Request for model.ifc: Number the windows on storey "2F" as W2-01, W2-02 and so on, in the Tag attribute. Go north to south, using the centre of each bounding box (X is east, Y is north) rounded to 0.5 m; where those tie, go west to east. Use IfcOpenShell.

First a look at what the model holds.

```python
import ifcopenshell
import ifcopenshell.util.element
import ifcopenshell.util.placement

model = ifcopenshell.open("model.ifc")
print(model.schema)
storey = next(s for s in model.by_type("IfcBuildingStorey") if s.Name == "2F")
windows = [e for e in ifcopenshell.util.element.get_decomposition(storey) if e.is_a("IfcWindow")]
for e in sorted(windows, key=lambda e: e.id()):
    origin = ifcopenshell.util.placement.get_local_placement(e.ObjectPlacement)[:3, 3]
    print(e.id(), e.Tag, e.Name, origin.round(2) + 0.0, sep=" | ")
```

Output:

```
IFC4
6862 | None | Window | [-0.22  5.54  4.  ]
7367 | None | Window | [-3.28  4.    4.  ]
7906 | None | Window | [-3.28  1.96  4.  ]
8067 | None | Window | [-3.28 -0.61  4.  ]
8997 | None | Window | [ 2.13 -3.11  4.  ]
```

```python
import ifcopenshell
import ifcopenshell.geom
import ifcopenshell.util.element
import ifcopenshell.util.shape

model = ifcopenshell.open("model.ifc")
settings = ifcopenshell.geom.settings()
settings.set("use-world-coords", True)


def centre(element):
    shape = ifcopenshell.geom.create_shape(settings, element)
    return ifcopenshell.util.shape.get_bbox_centroid(shape.geometry)


storey = next(s for s in model.by_type("IfcBuildingStorey") if s.Name == "2F")
windows = [e for e in ifcopenshell.util.element.get_decomposition(storey) if e.is_a("IfcWindow")]

# Insertion points can sit at a corner or the storey origin, so sort by the geometry (in metres).
centres = {e: centre(e) for e in windows}
windows.sort(key=lambda e: (-round(centres[e][1] / 0.5), centres[e][0]))

for i, e in enumerate(windows, start=1):
    number = f"W2-{i:02d}"
    e.Tag = number
    print(e.id(), number)

model.write("model_edited.ifc")
```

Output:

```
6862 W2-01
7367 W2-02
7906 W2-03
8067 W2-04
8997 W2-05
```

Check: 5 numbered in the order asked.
